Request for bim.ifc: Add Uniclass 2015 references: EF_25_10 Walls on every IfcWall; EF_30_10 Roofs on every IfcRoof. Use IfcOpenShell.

First a look at what the model holds.

```python
import ifcopenshell

model = ifcopenshell.open("bim.ifc")
print(model.schema)
print("classifications:", [c.Name for c in model.by_type("IfcClassification")])
for ifc_class in ("IfcDoor", "IfcRoof", "IfcStair", "IfcWall", "IfcWindow"):
    print(ifc_class, len(model.by_type(ifc_class)))
```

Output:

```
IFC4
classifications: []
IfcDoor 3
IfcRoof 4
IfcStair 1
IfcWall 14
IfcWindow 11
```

```python
import ifcopenshell
import ifcopenshell.api.classification

model = ifcopenshell.open("bim.ifc")

system = ifcopenshell.api.classification.add_classification(model, classification="Uniclass 2015")

codes = {
    "IfcWall": ("EF_25_10", "Walls"),
    "IfcRoof": ("EF_30_10", "Roofs"),
}
for ifc_class, (code, name) in codes.items():
    products = model.by_type(ifc_class)
    ifcopenshell.api.classification.add_reference(
        model, products=products, classification=system, identification=code, name=name
    )
    print(code, len(products))

model.write("bim_v2.ifc")
```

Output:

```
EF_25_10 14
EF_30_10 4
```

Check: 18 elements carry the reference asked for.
